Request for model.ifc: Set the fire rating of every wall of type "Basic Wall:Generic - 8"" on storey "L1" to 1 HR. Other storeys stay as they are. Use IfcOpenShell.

First a look at what the model holds.

```python
import ifcopenshell
import ifcopenshell.util.element

model = ifcopenshell.open("model.ifc")
print(model.schema)
storey = next(s for s in model.by_type("IfcBuildingStorey") if s.Name == "L1")
walls = [e for e in ifcopenshell.util.element.get_decomposition(storey) if e.is_a("IfcWall")]
seen = {}
for e in walls:
    element_type = ifcopenshell.util.element.get_type(e)
    key = (element_type.Name if element_type != e and element_type else None, ifcopenshell.util.element.get_pset(e, "Pset_WallCommon", "FireRating"))
    seen[key] = seen.get(key, 0) + 1
for (name, value), count in sorted(seen.items(), key=str):
    print(count, "x", name, "|", value)
```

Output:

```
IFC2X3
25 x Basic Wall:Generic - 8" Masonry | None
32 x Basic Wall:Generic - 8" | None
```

```python
import ifcopenshell
import ifcopenshell.api.pset
import ifcopenshell.util.element

model = ifcopenshell.open("model.ifc")

storey = next(s for s in model.by_type("IfcBuildingStorey") if s.Name == "L1")
walls = [e for e in ifcopenshell.util.element.get_decomposition(storey) if e.is_a("IfcWall")]

count = 0
for e in walls:
    element_type = ifcopenshell.util.element.get_type(e)
    if element_type in (None, e) or element_type.Name != 'Basic Wall:Generic - 8"':
        continue
    # add_pset returns the element's existing set when there is one.
    pset = ifcopenshell.api.pset.add_pset(model, product=e, name="Pset_WallCommon")
    ifcopenshell.api.pset.edit_pset(model, pset=pset, properties={"FireRating": "1 HR"})
    count += 1

print(count, "walls updated")

model.write("model_updated.ifc")
```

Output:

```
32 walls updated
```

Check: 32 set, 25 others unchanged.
